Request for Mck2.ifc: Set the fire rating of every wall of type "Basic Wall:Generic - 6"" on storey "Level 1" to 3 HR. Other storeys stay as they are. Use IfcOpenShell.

First a look at what the model holds.

```python
import ifcopenshell
import ifcopenshell.util.element

model = ifcopenshell.open("Mck2.ifc")
print(model.schema)
storey = next(s for s in model.by_type("IfcBuildingStorey") if s.Name == "Level 1")
walls = [e for e in ifcopenshell.util.element.get_decomposition(storey) if e.is_a("IfcWall")]
seen = {}
for e in walls:
    element_type = ifcopenshell.util.element.get_type(e)
    key = (element_type.Name if element_type != e and element_type else None, ifcopenshell.util.element.get_pset(e, "Pset_WallCommon", "FireRating"))
    seen[key] = seen.get(key, 0) + 1
for (name, value), count in sorted(seen.items(), key=str):
    print(count, "x", name, "|", value)
```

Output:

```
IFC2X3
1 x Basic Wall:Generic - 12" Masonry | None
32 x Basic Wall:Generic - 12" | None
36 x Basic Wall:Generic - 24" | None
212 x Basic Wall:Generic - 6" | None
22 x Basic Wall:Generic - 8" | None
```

```python
import ifcopenshell
import ifcopenshell.api.pset
import ifcopenshell.util.element

model = ifcopenshell.open("Mck2.ifc")

storey = next(s for s in model.by_type("IfcBuildingStorey") if s.Name == "Level 1")
walls = [e for e in ifcopenshell.util.element.get_decomposition(storey) if e.is_a("IfcWall")]

count = 0
for e in walls:
    element_type = ifcopenshell.util.element.get_type(e)
    if element_type in (None, e) or element_type.Name != 'Basic Wall:Generic - 6"':
        continue
    # add_pset returns the element's existing set when there is one.
    pset = ifcopenshell.api.pset.add_pset(model, product=e, name="Pset_WallCommon")
    ifcopenshell.api.pset.edit_pset(model, pset=pset, properties={"FireRating": "3 HR"})
    count += 1

print(count, "walls updated")

model.write("Mck2_v2.ifc")
```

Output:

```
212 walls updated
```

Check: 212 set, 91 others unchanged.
